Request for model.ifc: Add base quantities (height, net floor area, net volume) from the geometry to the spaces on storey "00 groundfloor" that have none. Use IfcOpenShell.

First a look at what the model holds.

```python
import ifcopenshell
import ifcopenshell.util.element
import ifcopenshell.util.unit

model = ifcopenshell.open("model.ifc")
print(model.schema)
for unit_type in ("LENGTHUNIT", "AREAUNIT", "VOLUMEUNIT"):
    print(unit_type, ifcopenshell.util.unit.calculate_unit_scale(model, unit_type))
storey = next(s for s in model.by_type("IfcBuildingStorey") if s.Name == "00 groundfloor")
spaces = [e for e in ifcopenshell.util.element.get_decomposition(storey) if e.is_a("IfcSpace")]
for e in sorted(spaces, key=lambda e: e.id()):
    print(e.id(), e.is_a(), e.Name, list(ifcopenshell.util.element.get_psets(e, qtos_only=True)), sep=" | ")
```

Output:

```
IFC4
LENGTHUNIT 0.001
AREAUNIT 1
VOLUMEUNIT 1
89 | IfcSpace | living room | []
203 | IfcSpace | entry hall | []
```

```python
import ifcopenshell
import ifcopenshell.api.pset
import ifcopenshell.geom
import ifcopenshell.util.element
import ifcopenshell.util.shape
import ifcopenshell.util.unit

model = ifcopenshell.open("model.ifc")
unit_scale = ifcopenshell.util.unit.calculate_unit_scale(model)
area_scale = ifcopenshell.util.unit.calculate_unit_scale(model, "AREAUNIT")
volume_scale = ifcopenshell.util.unit.calculate_unit_scale(model, "VOLUMEUNIT")
settings = ifcopenshell.geom.settings()

storey = next(s for s in model.by_type("IfcBuildingStorey") if s.Name == "00 groundfloor")
spaces = [e for e in ifcopenshell.util.element.get_decomposition(storey) if e.is_a("IfcSpace")]

for e in sorted(spaces, key=lambda e: e.id()):
    if ifcopenshell.util.element.get_psets(e, qtos_only=True, should_inherit=False):
        continue
    # Geometry comes back in metres, in the element's own axes.
    shape = ifcopenshell.geom.create_shape(settings, e)
    values = {
        "Height": ifcopenshell.util.shape.get_z(shape.geometry) / unit_scale,
        "NetFloorArea": ifcopenshell.util.shape.get_footprint_area(shape.geometry) / area_scale,
        "NetVolume": ifcopenshell.util.shape.get_volume(shape.geometry) / volume_scale,
    }
    qto = ifcopenshell.api.pset.add_qto(model, product=e, name="Qto_SpaceBaseQuantities")
    ifcopenshell.api.pset.edit_qto(model, qto=qto, properties=values)
    print(e.id(), {k: round(v, 3) for k, v in values.items()})

model.write("model_edited.ifc")
```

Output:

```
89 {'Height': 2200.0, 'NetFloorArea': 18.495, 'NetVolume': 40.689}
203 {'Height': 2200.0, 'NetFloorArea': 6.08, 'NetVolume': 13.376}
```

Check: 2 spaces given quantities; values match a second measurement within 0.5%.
